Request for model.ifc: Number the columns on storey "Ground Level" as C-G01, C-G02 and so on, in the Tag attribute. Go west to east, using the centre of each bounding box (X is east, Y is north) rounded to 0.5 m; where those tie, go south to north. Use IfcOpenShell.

First a look at what the model holds.

```python
import ifcopenshell
import ifcopenshell.util.element
import ifcopenshell.util.placement

model = ifcopenshell.open("model.ifc")
print(model.schema)
storey = next(s for s in model.by_type("IfcBuildingStorey") if s.Name == "Ground Level")
columns = [e for e in ifcopenshell.util.element.get_decomposition(storey) if e.is_a("IfcColumn")]
for e in sorted(columns, key=lambda e: e.id()):
    origin = ifcopenshell.util.placement.get_local_placement(e.ObjectPlacement)[:3, 3]
    print(e.id(), e.Tag, e.Name, origin.round(2) + 0.0, sep=" | ")
```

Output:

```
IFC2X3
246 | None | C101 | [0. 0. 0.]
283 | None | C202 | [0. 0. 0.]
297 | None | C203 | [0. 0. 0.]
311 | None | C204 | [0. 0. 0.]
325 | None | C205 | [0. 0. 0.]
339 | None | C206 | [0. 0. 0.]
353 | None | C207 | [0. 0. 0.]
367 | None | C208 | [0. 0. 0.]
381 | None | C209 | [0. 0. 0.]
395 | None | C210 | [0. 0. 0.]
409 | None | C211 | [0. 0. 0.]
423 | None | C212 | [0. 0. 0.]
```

```python
import ifcopenshell
import ifcopenshell.geom
import ifcopenshell.util.element
import ifcopenshell.util.shape

model = ifcopenshell.open("model.ifc")
settings = ifcopenshell.geom.settings()
settings.set("use-world-coords", True)


def centre(element):
    shape = ifcopenshell.geom.create_shape(settings, element)
    return ifcopenshell.util.shape.get_bbox_centroid(shape.geometry)


storey = next(s for s in model.by_type("IfcBuildingStorey") if s.Name == "Ground Level")
columns = [e for e in ifcopenshell.util.element.get_decomposition(storey) if e.is_a("IfcColumn")]

# Insertion points can sit at a corner or the storey origin, so sort by the geometry (in metres).
centres = {e: centre(e) for e in columns}
columns.sort(key=lambda e: (round(centres[e][0] / 0.5), centres[e][1]))

for i, e in enumerate(columns, start=1):
    number = f"C-G{i:02d}"
    e.Tag = number
    print(e.id(), number)

model.write("model_edited.ifc")
```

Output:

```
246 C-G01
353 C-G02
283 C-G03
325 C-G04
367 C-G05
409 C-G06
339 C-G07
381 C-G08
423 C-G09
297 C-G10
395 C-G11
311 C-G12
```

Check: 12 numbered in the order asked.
